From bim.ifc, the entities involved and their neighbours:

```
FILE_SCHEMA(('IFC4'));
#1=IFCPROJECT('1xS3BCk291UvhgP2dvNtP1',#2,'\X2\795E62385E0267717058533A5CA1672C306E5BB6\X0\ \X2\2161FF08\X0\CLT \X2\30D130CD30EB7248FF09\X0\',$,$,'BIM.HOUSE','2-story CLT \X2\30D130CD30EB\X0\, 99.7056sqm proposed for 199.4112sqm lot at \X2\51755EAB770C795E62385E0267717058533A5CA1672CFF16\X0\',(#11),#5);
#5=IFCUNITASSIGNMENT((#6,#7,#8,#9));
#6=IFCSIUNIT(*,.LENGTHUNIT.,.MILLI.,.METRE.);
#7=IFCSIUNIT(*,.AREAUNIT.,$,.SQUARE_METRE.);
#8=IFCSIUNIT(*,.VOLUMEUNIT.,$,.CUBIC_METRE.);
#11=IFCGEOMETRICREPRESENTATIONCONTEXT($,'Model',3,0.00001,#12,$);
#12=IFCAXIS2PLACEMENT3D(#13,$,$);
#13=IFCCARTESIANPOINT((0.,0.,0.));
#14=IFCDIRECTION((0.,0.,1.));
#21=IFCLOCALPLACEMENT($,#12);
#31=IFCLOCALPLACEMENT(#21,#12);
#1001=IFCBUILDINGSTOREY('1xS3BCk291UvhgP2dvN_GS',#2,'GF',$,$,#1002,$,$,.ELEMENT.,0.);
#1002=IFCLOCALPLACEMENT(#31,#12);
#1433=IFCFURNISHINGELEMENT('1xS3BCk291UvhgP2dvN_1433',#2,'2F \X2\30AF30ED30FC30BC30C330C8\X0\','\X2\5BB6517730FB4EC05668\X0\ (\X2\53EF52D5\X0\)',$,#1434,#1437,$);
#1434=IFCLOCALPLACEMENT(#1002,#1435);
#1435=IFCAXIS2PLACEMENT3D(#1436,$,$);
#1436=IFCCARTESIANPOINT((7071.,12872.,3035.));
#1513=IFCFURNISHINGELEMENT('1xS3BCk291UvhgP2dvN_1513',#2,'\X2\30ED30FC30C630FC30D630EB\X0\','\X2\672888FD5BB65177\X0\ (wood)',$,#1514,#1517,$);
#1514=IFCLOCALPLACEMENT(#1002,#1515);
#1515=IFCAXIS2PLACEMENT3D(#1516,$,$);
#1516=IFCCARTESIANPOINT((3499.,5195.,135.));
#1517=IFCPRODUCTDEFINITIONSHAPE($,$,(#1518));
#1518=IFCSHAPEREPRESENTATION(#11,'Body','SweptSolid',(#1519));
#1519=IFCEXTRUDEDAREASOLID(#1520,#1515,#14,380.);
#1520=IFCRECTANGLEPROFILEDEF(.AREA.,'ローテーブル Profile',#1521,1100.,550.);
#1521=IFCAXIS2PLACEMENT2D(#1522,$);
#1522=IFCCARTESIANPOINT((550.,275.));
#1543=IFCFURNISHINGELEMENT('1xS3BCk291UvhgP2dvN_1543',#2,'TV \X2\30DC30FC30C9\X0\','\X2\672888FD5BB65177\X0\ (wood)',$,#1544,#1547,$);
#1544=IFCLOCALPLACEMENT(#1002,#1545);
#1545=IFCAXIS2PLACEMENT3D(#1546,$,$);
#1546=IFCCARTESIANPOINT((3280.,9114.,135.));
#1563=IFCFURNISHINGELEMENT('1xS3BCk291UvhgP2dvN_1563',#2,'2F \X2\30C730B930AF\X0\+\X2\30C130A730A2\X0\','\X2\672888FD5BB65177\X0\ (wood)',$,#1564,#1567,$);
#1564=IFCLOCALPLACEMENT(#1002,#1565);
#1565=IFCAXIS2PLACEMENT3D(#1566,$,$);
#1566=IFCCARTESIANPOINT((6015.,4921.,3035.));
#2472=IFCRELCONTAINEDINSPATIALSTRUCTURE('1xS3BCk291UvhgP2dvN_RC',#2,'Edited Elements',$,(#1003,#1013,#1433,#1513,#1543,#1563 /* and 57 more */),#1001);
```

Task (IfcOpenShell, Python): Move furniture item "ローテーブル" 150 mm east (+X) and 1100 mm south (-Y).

```python
import ifcopenshell
import ifcopenshell.api.geometry
import ifcopenshell.util.placement

model = ifcopenshell.open("bim.ifc")

item = model.by_guid("1xS3BCk291UvhgP2dvN_1513")
matrix = ifcopenshell.util.placement.get_local_placement(item.ObjectPlacement)
matrix[0, 3] += 150.0
matrix[1, 3] -= 1100.0
ifcopenshell.api.geometry.edit_object_placement(model, product=item, matrix=matrix, is_si=False)

print(ifcopenshell.util.placement.get_local_placement(item.ObjectPlacement).round(3) + 0.0)

model.write("bim_updated.ifc")
```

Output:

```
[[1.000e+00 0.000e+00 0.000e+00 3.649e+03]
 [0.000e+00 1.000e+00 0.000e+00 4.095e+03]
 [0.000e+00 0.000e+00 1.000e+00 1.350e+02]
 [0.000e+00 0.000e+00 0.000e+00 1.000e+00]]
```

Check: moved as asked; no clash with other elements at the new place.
